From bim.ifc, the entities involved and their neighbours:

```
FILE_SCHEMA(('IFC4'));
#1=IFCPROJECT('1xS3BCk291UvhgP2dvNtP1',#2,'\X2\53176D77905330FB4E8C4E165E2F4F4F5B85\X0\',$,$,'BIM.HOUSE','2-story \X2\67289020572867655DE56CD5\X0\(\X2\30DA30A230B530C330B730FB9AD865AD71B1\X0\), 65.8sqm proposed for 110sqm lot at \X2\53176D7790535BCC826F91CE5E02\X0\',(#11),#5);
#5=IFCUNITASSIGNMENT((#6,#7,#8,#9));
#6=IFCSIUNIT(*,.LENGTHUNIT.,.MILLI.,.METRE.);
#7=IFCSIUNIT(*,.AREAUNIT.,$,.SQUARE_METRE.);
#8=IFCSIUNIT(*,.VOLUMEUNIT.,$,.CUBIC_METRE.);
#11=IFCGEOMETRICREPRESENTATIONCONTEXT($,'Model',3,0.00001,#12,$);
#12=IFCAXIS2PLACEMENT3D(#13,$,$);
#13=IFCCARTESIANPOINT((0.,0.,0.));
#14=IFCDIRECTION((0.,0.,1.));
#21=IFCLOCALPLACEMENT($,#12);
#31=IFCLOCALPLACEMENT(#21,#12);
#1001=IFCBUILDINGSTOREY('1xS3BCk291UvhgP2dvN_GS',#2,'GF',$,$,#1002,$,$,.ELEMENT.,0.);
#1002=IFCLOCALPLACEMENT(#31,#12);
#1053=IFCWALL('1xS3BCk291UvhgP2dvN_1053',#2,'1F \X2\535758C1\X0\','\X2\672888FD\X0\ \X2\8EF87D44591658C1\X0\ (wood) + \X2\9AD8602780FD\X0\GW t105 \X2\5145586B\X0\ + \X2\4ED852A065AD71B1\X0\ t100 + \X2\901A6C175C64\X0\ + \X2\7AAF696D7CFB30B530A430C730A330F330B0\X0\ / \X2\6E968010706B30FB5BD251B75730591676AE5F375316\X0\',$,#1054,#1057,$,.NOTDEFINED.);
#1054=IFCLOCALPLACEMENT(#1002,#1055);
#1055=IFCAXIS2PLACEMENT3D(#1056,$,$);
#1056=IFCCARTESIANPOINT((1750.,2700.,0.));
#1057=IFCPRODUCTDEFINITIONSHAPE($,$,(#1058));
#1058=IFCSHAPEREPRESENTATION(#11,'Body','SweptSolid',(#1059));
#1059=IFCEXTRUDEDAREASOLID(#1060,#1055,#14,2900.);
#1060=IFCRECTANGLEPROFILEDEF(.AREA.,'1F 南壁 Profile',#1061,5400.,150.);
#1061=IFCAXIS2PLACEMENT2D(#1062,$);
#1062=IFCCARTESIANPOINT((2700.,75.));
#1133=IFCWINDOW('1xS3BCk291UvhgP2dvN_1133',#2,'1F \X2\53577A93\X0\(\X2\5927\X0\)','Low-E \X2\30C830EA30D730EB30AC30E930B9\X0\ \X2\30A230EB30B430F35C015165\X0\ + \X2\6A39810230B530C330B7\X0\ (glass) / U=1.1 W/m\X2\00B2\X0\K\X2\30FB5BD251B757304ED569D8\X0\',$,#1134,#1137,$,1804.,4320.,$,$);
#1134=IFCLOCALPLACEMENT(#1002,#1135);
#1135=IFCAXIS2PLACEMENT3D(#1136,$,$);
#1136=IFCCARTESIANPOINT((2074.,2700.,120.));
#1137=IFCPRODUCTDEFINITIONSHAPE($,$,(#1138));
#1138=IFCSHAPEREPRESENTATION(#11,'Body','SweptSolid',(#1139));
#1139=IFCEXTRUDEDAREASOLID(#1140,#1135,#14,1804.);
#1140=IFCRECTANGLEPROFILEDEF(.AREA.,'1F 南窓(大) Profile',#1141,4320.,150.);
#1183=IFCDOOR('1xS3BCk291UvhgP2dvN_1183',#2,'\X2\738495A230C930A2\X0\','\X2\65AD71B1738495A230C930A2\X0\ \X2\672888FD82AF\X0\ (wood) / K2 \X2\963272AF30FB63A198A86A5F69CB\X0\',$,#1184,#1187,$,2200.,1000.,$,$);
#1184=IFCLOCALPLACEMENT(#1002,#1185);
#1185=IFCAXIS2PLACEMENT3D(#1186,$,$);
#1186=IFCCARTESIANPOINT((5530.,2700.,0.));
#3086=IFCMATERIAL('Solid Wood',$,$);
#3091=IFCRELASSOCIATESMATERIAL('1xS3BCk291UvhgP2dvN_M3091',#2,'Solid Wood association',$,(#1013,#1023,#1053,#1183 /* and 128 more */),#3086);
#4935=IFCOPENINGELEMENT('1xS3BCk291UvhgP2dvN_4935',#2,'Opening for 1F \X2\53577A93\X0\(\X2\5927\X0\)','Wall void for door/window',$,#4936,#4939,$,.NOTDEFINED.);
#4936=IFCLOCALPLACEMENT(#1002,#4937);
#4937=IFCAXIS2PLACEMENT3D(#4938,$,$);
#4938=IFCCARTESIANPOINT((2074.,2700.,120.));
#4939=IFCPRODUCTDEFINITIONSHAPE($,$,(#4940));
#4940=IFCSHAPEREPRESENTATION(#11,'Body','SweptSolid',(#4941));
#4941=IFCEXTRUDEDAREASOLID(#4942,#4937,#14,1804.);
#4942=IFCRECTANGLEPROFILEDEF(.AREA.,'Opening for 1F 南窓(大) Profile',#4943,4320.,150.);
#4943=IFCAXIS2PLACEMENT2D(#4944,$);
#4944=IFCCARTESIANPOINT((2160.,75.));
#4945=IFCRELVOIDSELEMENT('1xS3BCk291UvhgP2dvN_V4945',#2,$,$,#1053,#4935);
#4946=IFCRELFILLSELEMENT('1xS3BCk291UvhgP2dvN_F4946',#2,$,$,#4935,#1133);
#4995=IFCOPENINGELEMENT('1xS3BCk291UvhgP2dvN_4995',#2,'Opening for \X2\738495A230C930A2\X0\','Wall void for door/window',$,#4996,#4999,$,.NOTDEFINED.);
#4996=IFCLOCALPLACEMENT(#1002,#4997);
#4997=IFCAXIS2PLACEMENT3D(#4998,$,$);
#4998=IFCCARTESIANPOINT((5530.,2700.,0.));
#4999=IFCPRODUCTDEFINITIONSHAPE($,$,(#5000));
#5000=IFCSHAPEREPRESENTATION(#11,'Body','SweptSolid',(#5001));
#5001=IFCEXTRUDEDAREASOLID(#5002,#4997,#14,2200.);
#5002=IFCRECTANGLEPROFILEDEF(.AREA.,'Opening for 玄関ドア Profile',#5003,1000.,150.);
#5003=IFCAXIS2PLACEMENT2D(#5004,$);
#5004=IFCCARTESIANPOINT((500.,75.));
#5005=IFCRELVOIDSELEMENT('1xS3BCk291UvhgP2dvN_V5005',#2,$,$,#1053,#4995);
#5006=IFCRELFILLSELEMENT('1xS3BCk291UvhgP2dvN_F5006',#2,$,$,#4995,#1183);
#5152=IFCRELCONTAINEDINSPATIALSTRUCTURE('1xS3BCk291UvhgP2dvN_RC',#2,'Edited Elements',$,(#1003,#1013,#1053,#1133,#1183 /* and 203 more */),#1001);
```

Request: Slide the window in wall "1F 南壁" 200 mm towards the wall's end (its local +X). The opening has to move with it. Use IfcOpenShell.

```python
import ifcopenshell
import ifcopenshell.api.geometry
import ifcopenshell.util.placement
import ifcopenshell.util.unit

model = ifcopenshell.open("bim.ifc")
unit_scale = ifcopenshell.util.unit.calculate_unit_scale(model)

window = model.by_guid("1xS3BCk291UvhgP2dvN_1133")
opening = window.FillsVoids[0].RelatingOpeningElement
wall = opening.VoidsElements[0].RelatingBuildingElement

wall_matrix = ifcopenshell.util.placement.get_local_placement(wall.ObjectPlacement)
shift = wall_matrix[:3, 0] * 0.2 / unit_scale
before = ifcopenshell.util.placement.get_local_placement(window.ObjectPlacement)[:3, 3].copy()

# The window is not placed relative to its opening, so move both.
for product in (opening, window):
    matrix = ifcopenshell.util.placement.get_local_placement(product.ObjectPlacement)
    matrix[:3, 3] += shift
    ifcopenshell.api.geometry.edit_object_placement(model, product=product, matrix=matrix, is_si=False)

after = ifcopenshell.util.placement.get_local_placement(window.ObjectPlacement)[:3, 3]
print("window moved by", (after - before).round(3) + 0.0)

model.write("bim_updated.ifc")
```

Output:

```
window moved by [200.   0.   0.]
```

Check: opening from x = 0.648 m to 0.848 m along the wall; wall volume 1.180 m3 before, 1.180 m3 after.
